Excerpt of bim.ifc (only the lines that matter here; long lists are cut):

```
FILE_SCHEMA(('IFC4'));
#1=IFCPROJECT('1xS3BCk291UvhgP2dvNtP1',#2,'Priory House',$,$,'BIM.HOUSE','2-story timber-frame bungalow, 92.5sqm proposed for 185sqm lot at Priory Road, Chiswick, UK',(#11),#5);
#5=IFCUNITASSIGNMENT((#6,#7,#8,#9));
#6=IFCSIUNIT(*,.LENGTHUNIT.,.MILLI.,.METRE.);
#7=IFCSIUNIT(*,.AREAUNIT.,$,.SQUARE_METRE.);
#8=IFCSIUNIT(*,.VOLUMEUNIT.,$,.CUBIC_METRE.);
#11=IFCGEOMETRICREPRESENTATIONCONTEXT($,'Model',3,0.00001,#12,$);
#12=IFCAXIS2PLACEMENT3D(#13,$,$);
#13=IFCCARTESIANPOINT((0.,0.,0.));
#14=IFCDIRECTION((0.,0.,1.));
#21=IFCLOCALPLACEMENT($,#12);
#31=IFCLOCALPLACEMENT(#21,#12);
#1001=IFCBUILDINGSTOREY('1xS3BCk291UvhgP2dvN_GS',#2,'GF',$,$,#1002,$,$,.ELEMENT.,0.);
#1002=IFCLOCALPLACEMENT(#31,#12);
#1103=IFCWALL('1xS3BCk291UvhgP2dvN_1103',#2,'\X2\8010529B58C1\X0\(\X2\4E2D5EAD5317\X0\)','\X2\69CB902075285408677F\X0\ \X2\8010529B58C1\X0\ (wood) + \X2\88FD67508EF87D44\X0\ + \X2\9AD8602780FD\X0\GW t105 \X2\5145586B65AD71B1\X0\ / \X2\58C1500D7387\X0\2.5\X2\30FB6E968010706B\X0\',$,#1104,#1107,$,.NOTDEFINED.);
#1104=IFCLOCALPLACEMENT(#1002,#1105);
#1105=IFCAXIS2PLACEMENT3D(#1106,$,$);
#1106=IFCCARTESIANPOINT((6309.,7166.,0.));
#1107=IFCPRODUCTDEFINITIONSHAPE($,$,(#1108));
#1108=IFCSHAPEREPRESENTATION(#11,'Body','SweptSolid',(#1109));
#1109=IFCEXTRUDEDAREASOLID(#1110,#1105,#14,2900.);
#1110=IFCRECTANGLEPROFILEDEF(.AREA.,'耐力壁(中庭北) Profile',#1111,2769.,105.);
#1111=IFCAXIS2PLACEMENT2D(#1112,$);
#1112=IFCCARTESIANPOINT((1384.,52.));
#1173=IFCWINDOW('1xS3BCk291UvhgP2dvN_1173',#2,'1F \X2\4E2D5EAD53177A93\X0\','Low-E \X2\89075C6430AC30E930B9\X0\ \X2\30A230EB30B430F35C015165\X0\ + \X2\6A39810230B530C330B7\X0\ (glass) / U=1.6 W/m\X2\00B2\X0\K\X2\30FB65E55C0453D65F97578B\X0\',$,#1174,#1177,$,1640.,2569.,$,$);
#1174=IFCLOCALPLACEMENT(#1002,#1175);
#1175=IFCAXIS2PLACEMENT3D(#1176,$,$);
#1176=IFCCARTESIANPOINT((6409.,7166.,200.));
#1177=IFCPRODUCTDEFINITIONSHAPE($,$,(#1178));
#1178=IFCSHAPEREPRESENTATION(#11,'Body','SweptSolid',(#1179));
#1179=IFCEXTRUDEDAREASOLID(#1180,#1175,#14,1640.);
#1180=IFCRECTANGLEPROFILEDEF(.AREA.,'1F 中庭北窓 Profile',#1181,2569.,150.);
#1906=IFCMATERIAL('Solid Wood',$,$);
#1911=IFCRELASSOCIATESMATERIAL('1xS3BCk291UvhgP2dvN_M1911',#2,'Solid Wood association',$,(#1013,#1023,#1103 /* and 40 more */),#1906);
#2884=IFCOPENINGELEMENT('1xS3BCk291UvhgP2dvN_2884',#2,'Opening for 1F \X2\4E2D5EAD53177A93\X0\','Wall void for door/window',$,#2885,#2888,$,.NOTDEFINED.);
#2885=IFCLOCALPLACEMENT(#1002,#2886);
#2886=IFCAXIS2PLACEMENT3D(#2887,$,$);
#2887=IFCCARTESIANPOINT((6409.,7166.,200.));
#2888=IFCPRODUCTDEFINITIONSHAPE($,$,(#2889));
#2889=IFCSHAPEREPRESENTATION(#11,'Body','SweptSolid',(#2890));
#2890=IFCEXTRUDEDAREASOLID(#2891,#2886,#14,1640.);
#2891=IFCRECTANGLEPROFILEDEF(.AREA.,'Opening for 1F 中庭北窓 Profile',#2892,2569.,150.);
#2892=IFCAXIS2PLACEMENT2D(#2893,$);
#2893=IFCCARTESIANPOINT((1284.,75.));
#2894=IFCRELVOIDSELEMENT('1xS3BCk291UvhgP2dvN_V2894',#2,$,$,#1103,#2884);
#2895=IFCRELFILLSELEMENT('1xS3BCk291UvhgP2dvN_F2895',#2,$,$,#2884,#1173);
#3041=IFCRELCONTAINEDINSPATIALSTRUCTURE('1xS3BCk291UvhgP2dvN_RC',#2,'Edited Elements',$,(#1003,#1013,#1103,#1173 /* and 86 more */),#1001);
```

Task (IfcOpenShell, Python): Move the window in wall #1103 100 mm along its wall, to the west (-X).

```python
import ifcopenshell
import ifcopenshell.api.geometry
import ifcopenshell.util.placement

model = ifcopenshell.open("bim.ifc")

window = model.by_guid("1xS3BCk291UvhgP2dvN_1173")
opening = window.FillsVoids[0].RelatingOpeningElement
wall = opening.VoidsElements[0].RelatingBuildingElement

wall_matrix = ifcopenshell.util.placement.get_local_placement(wall.ObjectPlacement)
shift = wall_matrix[:3, 0] * -100.0
before = ifcopenshell.util.placement.get_local_placement(window.ObjectPlacement)[:3, 3].copy()

# The window is not placed relative to its opening, so move both.
for product in (opening, window):
    matrix = ifcopenshell.util.placement.get_local_placement(product.ObjectPlacement)
    matrix[:3, 3] += shift
    ifcopenshell.api.geometry.edit_object_placement(model, product=product, matrix=matrix, is_si=False)

after = ifcopenshell.util.placement.get_local_placement(window.ObjectPlacement)[:3, 3]
print("window moved by", (after - before).round(3) + 0.0)

model.write("bim-out.ifc")
```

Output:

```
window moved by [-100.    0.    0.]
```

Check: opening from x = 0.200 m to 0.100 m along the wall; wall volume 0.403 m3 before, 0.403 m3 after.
